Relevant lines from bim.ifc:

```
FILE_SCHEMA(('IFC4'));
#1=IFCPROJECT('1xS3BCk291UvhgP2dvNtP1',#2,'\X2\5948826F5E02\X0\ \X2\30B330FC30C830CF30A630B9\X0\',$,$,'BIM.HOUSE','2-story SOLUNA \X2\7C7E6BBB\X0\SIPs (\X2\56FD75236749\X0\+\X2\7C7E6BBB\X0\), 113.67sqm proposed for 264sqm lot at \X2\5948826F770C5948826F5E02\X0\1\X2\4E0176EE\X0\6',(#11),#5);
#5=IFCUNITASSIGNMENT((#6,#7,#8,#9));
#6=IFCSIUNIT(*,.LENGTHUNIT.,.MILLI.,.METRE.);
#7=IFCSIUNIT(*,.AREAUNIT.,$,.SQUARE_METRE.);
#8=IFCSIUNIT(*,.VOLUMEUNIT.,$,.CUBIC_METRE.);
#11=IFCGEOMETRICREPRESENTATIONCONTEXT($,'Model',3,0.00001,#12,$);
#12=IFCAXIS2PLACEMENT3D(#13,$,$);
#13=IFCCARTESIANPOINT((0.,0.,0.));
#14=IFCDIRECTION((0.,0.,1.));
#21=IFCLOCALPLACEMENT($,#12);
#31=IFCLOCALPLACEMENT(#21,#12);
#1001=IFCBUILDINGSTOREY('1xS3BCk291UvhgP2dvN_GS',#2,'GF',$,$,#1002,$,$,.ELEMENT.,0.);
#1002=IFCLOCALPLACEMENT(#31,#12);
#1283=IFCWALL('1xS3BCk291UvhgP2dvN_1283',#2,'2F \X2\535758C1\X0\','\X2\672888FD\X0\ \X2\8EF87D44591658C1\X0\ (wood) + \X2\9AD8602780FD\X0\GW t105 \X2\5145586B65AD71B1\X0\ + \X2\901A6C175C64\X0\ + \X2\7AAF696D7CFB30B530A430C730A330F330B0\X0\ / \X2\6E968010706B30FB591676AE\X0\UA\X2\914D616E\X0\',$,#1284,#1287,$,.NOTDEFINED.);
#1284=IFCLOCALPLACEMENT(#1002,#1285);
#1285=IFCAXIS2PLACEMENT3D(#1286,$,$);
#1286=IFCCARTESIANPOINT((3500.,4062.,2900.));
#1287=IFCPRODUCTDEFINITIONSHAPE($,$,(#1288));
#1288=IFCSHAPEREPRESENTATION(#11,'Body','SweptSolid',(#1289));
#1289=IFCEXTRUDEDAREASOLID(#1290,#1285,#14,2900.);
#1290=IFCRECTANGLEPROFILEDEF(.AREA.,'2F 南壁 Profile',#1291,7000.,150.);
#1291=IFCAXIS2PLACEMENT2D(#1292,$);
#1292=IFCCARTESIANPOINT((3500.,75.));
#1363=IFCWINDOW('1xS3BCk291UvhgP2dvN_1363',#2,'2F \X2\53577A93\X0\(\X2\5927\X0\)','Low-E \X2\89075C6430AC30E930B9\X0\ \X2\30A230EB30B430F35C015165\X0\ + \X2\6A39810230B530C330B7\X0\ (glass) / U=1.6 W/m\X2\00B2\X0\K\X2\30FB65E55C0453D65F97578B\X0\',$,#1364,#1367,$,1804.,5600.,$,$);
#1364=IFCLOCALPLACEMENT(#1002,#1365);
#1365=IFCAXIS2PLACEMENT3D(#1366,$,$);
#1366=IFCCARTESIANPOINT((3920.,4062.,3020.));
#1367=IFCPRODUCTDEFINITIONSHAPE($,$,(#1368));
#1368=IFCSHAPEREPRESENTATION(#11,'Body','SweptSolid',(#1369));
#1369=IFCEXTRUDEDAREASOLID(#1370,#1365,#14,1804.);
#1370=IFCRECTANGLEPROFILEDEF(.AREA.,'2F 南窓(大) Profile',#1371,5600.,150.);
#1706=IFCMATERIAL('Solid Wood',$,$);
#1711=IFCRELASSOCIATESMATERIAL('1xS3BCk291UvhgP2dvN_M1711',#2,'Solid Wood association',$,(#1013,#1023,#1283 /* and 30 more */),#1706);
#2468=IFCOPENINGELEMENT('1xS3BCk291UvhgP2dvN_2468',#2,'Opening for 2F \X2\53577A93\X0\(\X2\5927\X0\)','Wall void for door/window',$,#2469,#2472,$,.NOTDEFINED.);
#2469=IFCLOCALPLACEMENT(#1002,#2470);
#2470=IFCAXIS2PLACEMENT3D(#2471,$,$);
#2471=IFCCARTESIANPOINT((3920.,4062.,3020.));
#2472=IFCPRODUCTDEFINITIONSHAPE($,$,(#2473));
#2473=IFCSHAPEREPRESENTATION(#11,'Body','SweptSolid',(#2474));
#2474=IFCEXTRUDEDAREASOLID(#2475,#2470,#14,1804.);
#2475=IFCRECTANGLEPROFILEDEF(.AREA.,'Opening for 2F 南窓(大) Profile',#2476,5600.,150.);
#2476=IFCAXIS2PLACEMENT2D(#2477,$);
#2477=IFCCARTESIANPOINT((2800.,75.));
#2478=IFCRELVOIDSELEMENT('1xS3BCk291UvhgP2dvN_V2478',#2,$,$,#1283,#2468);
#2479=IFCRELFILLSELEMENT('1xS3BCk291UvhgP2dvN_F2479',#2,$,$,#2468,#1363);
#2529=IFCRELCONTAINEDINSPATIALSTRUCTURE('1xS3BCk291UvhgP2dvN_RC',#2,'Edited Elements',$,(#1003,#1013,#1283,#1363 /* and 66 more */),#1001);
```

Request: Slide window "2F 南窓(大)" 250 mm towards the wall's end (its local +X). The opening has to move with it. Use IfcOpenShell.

```python
import ifcopenshell
import ifcopenshell.api.geometry
import ifcopenshell.util.placement
import ifcopenshell.util.unit

model = ifcopenshell.open("bim.ifc")
unit_scale = ifcopenshell.util.unit.calculate_unit_scale(model)

window = model.by_id(1363)
opening = window.FillsVoids[0].RelatingOpeningElement
wall = opening.VoidsElements[0].RelatingBuildingElement

wall_matrix = ifcopenshell.util.placement.get_local_placement(wall.ObjectPlacement)
shift = wall_matrix[:3, 0] * 0.25 / unit_scale
before = ifcopenshell.util.placement.get_local_placement(window.ObjectPlacement)[:3, 3].copy()

# The window is not placed relative to its opening, so move both.
for product in (opening, window):
    matrix = ifcopenshell.util.placement.get_local_placement(product.ObjectPlacement)
    matrix[:3, 3] += shift
    ifcopenshell.api.geometry.edit_object_placement(model, product=product, matrix=matrix, is_si=False)

after = ifcopenshell.util.placement.get_local_placement(window.ObjectPlacement)[:3, 3]
print("window moved by", (after - before).round(3) + 0.0)

model.write("bim_updated.ifc")
```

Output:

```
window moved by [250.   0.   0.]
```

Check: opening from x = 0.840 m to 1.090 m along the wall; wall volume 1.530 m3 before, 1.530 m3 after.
